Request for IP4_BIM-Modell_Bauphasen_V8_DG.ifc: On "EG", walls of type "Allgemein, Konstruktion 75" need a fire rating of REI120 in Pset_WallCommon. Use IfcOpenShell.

First a look at what the model holds.

```python
import ifcopenshell
import ifcopenshell.util.element

model = ifcopenshell.open("IP4_BIM-Modell_Bauphasen_V8_DG.ifc")
print(model.schema)
storey = next(s for s in model.by_type("IfcBuildingStorey") if s.Name == "EG")
walls = [e for e in ifcopenshell.util.element.get_decomposition(storey) if e.is_a("IfcWall")]
seen = {}
for e in walls:
    element_type = ifcopenshell.util.element.get_type(e)
    key = (element_type.Name if element_type != e and element_type else None, ifcopenshell.util.element.get_pset(e, "Pset_WallCommon", "FireRating"))
    seen[key] = seen.get(key, 0) + 1
for (name, value), count in sorted(seen.items(), key=str):
    print(count, "x", name, "|", value)
```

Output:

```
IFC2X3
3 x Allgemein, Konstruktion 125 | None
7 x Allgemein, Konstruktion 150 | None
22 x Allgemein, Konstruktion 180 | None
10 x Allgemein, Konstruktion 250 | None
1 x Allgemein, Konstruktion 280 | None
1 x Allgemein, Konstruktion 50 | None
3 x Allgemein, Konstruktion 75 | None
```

```python
import ifcopenshell
import ifcopenshell.api.pset
import ifcopenshell.util.element

model = ifcopenshell.open("IP4_BIM-Modell_Bauphasen_V8_DG.ifc")

storey = next(s for s in model.by_type("IfcBuildingStorey") if s.Name == "EG")
walls = [e for e in ifcopenshell.util.element.get_decomposition(storey) if e.is_a("IfcWall")]

count = 0
for e in walls:
    element_type = ifcopenshell.util.element.get_type(e)
    if element_type in (None, e) or element_type.Name != "Allgemein, Konstruktion 75":
        continue
    # add_pset returns the element's existing set when there is one.
    pset = ifcopenshell.api.pset.add_pset(model, product=e, name="Pset_WallCommon")
    ifcopenshell.api.pset.edit_pset(model, pset=pset, properties={"FireRating": "REI120"})
    count += 1

print(count, "walls updated")

model.write("IP4_BIM-Modell_Bauphasen_V8_DG_rev.ifc")
```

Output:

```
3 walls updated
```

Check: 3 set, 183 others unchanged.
